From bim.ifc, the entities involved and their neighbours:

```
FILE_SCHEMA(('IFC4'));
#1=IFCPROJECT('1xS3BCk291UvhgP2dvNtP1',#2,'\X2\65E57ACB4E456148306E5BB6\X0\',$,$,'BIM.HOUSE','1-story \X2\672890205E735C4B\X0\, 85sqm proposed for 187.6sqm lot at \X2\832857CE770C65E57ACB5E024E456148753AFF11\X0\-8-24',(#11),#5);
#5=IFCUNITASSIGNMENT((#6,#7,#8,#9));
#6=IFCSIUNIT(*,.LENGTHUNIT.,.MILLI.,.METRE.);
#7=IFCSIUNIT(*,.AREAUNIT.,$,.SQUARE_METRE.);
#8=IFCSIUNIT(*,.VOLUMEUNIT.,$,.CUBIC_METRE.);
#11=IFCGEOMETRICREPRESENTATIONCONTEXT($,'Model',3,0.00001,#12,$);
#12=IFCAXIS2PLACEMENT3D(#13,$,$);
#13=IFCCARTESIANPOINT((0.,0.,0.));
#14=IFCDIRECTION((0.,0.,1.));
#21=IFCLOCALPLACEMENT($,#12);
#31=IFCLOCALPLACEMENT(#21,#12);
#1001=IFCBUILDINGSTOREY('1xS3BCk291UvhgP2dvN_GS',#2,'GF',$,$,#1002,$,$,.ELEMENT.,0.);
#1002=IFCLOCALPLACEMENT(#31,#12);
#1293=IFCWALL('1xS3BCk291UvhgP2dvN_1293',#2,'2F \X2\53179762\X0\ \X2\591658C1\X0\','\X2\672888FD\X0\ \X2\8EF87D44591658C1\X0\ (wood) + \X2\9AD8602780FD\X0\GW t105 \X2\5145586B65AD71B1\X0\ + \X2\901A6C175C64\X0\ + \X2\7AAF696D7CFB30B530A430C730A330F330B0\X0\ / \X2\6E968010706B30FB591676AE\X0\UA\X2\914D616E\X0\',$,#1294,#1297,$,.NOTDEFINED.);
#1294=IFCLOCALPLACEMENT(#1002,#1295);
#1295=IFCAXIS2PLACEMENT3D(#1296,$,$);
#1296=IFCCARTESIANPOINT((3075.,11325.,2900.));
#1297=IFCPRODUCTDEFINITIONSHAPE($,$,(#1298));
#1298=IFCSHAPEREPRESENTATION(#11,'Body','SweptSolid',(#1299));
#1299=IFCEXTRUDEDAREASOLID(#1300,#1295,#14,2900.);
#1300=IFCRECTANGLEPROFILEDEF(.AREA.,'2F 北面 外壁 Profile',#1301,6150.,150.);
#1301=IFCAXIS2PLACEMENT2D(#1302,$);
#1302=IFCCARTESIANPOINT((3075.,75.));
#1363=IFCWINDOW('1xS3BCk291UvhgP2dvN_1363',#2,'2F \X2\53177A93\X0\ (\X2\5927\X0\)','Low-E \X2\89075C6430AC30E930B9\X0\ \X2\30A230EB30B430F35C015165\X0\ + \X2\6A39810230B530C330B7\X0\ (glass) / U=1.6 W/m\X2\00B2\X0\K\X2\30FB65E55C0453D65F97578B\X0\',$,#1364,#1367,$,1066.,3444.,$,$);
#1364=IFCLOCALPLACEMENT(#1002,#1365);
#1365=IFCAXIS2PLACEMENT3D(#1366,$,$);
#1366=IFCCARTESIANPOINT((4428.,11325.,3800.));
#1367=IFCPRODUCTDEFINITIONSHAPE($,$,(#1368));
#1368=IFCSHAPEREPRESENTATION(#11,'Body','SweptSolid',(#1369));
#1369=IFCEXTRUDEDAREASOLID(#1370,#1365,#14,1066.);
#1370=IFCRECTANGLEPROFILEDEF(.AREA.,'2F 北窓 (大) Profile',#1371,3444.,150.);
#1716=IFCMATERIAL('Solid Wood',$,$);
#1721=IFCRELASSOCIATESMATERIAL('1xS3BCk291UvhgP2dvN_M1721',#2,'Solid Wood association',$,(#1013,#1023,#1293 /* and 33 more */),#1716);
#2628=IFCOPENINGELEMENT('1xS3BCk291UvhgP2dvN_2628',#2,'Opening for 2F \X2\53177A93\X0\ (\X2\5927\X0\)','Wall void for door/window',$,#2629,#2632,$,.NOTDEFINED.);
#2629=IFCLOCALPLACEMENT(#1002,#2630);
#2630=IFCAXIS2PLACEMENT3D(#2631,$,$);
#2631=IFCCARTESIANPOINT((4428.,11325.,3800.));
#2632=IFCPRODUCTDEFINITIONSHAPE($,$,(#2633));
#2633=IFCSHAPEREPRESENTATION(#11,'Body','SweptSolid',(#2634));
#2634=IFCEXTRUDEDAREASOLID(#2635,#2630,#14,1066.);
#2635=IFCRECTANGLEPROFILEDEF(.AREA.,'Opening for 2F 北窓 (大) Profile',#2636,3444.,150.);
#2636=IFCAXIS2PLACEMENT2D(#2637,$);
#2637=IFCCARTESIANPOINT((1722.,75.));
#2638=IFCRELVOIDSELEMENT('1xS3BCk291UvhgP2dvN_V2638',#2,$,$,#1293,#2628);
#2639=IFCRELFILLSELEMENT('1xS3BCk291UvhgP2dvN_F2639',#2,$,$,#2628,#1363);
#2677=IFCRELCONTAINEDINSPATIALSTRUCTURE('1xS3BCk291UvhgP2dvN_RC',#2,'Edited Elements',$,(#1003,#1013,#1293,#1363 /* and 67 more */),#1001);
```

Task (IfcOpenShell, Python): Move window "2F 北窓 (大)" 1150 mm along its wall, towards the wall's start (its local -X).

```python
import ifcopenshell
import ifcopenshell.api.geometry
import ifcopenshell.util.placement
import ifcopenshell.util.unit

model = ifcopenshell.open("bim.ifc")
unit_scale = ifcopenshell.util.unit.calculate_unit_scale(model)

window = model.by_guid("1xS3BCk291UvhgP2dvN_1363")
opening = window.FillsVoids[0].RelatingOpeningElement
wall = opening.VoidsElements[0].RelatingBuildingElement

wall_matrix = ifcopenshell.util.placement.get_local_placement(wall.ObjectPlacement)
shift = wall_matrix[:3, 0] * -1.15 / unit_scale
before = ifcopenshell.util.placement.get_local_placement(window.ObjectPlacement)[:3, 3].copy()

# The window is not placed relative to its opening, so move both.
for product in (opening, window):
    matrix = ifcopenshell.util.placement.get_local_placement(product.ObjectPlacement)
    matrix[:3, 3] += shift
    ifcopenshell.api.geometry.edit_object_placement(model, product=product, matrix=matrix, is_si=False)

after = ifcopenshell.util.placement.get_local_placement(window.ObjectPlacement)[:3, 3]
print("window moved by", (after - before).round(3) + 0.0)

model.write("bim_v2.ifc")
```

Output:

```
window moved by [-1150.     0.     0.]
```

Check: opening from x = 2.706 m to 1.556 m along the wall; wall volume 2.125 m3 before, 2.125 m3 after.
